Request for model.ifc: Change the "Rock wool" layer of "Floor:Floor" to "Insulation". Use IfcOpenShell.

First a look at what the model holds.

```python
import ifcopenshell
import ifcopenshell.util.element

model = ifcopenshell.open("model.ifc")
print(model.schema)
for layer_set in model.by_type("IfcMaterialLayerSet"):
    if layer_set.LayerSetName == "Floor:Floor":
        for layer in layer_set.MaterialLayers:
            print(layer.id(), layer.Material and layer.Material.Name, layer.LayerThickness, sep=" | ")
        print(len(ifcopenshell.util.element.get_elements_by_material(model, layer_set)), "elements and types use it")
print(sorted(m.Name for m in model.by_type("IfcMaterial") if m.Name)[:60])
```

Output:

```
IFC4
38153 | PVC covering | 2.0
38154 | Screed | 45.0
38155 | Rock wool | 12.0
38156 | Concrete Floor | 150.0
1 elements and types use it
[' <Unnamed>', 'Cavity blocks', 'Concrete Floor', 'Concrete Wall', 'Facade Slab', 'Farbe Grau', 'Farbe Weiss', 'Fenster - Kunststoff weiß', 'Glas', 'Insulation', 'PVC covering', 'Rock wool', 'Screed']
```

```python
import ifcopenshell
import ifcopenshell.api.material

model = ifcopenshell.open("model.ifc")

layer_set = next(s for s in model.by_type("IfcMaterialLayerSet") if s.LayerSetName == "Floor:Floor")
layer = next(l for l in layer_set.MaterialLayers if l.Material and l.Material.Name == "Rock wool")
material = next(m for m in model.by_type("IfcMaterial") if m.Name == "Insulation")

# Point this one layer at the other material; renaming the old one would change it everywhere.
ifcopenshell.api.material.edit_layer(model, layer=layer, attributes={}, material=material)

print([l.Material.Name if l.Material else None for l in layer_set.MaterialLayers])

model.write("model_v2.ifc")
```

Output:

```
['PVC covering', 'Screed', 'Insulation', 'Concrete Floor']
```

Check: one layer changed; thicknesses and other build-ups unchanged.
